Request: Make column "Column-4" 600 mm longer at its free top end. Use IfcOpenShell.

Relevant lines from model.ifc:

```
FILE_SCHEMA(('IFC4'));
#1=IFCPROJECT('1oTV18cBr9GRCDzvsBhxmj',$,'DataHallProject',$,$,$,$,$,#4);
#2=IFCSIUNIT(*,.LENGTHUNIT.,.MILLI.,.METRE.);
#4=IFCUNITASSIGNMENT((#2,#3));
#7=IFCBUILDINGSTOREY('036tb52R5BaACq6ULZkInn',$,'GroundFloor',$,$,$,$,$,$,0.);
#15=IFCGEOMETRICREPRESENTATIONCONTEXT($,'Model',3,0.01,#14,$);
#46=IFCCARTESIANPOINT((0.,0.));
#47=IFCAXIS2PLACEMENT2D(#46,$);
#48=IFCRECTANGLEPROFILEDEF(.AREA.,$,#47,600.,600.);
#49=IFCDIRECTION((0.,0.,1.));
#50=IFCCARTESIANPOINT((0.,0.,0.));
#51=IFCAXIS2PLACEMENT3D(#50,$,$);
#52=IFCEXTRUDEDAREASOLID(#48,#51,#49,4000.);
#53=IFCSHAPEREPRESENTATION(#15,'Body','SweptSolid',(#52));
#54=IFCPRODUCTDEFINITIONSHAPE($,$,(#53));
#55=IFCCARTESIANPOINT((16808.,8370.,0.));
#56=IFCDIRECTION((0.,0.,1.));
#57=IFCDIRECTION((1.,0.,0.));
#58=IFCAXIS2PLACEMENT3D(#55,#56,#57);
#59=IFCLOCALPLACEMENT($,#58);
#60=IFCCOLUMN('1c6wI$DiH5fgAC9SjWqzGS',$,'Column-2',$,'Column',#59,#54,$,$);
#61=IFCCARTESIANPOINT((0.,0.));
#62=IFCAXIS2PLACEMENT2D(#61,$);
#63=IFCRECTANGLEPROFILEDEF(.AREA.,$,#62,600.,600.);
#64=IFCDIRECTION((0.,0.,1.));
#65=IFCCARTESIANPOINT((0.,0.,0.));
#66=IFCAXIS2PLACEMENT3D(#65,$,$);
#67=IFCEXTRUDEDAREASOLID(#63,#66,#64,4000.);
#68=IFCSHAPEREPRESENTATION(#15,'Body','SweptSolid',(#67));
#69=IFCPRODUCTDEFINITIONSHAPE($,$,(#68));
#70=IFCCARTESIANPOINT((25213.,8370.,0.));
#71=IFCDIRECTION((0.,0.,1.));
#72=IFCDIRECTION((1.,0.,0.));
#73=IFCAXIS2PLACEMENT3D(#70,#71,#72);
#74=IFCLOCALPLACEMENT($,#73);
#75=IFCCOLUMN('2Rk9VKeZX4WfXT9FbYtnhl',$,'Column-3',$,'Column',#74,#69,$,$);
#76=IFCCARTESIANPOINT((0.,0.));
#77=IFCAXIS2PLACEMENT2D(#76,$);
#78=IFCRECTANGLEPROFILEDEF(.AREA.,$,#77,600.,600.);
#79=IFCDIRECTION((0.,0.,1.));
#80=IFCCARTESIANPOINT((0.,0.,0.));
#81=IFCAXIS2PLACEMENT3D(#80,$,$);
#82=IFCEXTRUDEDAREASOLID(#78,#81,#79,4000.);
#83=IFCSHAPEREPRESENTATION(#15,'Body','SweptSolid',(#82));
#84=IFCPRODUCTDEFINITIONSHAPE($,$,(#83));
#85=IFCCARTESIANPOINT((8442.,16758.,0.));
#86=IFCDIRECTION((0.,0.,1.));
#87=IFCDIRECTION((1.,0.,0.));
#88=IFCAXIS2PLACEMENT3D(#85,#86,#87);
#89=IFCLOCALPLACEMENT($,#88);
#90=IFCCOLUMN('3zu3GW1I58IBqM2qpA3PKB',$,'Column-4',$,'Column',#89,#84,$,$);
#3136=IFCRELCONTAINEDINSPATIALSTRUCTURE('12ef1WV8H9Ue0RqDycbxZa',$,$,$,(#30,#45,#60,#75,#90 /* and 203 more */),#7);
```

```python
import ifcopenshell
import ifcopenshell.util.unit

model = ifcopenshell.open("model.ifc")
unit_scale = ifcopenshell.util.unit.calculate_unit_scale(model)

member = model.by_guid("3zu3GW1I58IBqM2qpA3PKB")
change = 0.6 / unit_scale

# The extrusion runs towards the end named, so only its depth changes.
body = next(r for r in member.Representation.Representations if r.RepresentationIdentifier == "Body")
solid = body.Items[0]
old_length = solid.Depth
solid.Depth += change

print(f"length {old_length:g} -> {solid.Depth:g}")

model.write("model-out.ifc")
```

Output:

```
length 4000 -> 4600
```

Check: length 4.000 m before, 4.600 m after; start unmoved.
